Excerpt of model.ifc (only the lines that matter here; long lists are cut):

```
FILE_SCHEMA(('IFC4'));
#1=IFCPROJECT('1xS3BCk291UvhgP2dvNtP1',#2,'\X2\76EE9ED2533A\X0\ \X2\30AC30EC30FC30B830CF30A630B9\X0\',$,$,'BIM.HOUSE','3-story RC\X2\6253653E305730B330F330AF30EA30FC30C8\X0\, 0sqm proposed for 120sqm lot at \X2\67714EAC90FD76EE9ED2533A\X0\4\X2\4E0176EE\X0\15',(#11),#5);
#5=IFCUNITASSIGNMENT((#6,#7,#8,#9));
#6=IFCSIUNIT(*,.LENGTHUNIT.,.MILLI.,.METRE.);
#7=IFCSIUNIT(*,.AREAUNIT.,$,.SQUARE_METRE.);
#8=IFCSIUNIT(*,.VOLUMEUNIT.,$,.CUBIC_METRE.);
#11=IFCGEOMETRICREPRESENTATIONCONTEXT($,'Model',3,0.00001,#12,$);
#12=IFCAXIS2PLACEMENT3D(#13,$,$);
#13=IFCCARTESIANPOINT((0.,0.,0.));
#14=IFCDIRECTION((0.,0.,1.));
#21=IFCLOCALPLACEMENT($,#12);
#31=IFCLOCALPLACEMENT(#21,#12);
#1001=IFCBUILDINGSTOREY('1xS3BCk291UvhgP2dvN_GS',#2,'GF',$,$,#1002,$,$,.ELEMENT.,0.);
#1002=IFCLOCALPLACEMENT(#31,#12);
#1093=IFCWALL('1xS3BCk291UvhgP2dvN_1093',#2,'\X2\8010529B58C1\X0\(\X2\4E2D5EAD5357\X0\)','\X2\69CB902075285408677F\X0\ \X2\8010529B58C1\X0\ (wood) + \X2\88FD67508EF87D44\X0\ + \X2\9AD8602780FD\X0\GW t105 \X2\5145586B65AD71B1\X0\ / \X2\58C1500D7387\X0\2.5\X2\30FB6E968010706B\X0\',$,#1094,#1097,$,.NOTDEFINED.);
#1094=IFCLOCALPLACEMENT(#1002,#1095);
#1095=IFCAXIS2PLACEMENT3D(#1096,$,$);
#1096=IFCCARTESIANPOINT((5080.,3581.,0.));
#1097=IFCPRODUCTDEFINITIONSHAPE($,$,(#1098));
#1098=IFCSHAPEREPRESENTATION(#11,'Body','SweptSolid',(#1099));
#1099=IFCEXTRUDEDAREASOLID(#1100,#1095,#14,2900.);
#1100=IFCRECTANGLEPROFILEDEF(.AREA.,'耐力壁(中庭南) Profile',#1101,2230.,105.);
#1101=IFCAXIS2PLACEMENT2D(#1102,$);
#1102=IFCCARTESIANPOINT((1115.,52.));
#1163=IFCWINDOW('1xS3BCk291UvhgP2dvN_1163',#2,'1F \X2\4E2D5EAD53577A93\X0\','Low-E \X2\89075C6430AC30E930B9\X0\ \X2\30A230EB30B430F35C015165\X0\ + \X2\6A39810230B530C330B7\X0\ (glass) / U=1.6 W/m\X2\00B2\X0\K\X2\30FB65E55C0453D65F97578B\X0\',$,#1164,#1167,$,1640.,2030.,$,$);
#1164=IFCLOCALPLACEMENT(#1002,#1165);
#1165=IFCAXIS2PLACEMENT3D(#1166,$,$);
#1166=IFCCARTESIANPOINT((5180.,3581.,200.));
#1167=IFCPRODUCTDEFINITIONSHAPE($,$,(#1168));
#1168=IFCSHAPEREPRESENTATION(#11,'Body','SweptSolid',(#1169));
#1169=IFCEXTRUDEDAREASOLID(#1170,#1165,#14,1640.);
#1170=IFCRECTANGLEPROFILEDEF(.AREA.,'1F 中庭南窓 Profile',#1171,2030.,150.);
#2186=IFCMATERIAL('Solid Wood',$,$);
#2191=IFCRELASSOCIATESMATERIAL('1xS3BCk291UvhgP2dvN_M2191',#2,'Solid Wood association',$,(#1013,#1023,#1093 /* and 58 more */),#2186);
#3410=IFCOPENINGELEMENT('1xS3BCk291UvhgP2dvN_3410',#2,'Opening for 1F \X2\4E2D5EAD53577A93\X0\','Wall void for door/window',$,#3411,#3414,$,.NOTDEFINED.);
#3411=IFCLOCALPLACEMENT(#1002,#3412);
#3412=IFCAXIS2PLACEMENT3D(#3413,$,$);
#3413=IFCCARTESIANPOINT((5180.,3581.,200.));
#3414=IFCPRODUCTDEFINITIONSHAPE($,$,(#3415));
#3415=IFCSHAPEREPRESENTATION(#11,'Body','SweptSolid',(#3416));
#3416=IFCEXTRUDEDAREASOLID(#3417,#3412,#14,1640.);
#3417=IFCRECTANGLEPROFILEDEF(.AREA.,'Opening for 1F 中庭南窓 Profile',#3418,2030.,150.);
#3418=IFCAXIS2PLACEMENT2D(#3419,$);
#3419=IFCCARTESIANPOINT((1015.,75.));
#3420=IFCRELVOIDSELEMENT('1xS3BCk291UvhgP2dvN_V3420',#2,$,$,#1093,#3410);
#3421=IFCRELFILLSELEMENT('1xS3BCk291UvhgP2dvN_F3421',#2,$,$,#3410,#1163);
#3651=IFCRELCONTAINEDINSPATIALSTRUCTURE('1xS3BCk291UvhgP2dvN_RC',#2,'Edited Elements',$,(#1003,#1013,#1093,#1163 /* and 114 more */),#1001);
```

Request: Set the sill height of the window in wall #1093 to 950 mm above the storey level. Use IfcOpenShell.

```python
import numpy as np
import ifcopenshell
import ifcopenshell.api.geometry
import ifcopenshell.geom
import ifcopenshell.util.element
import ifcopenshell.util.placement
import ifcopenshell.util.shape
import ifcopenshell.util.unit

model = ifcopenshell.open("model.ifc")
unit_scale = ifcopenshell.util.unit.calculate_unit_scale(model)

window = model.by_guid("1xS3BCk291UvhgP2dvN_1163")
opening = window.FillsVoids[0].RelatingOpeningElement
storey = ifcopenshell.util.element.get_container(window, ifc_class="IfcBuildingStorey")
level = ifcopenshell.util.placement.get_local_placement(storey.ObjectPlacement)[2, 3]

# The opening's origin need not be at the sill, so measure its lowest point.
shape = ifcopenshell.geom.create_shape(ifcopenshell.geom.settings(), opening)
bottom = ifcopenshell.util.shape.get_shape_bottom_elevation(shape, shape.geometry) / unit_scale
dz = level + 0.95 / unit_scale - bottom

shift = np.array([0.0, 0.0, dz])
# The window is not placed relative to its opening, so move both.
for product in (opening, window):
    matrix = ifcopenshell.util.placement.get_local_placement(product.ObjectPlacement)
    matrix[:3, 3] += shift
    ifcopenshell.api.geometry.edit_object_placement(model, product=product, matrix=matrix, is_si=False)

print(f"moved by {dz * unit_scale:+.3f} m")

model.write("model-out.ifc")
```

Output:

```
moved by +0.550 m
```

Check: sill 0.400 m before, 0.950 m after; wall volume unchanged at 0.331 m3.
